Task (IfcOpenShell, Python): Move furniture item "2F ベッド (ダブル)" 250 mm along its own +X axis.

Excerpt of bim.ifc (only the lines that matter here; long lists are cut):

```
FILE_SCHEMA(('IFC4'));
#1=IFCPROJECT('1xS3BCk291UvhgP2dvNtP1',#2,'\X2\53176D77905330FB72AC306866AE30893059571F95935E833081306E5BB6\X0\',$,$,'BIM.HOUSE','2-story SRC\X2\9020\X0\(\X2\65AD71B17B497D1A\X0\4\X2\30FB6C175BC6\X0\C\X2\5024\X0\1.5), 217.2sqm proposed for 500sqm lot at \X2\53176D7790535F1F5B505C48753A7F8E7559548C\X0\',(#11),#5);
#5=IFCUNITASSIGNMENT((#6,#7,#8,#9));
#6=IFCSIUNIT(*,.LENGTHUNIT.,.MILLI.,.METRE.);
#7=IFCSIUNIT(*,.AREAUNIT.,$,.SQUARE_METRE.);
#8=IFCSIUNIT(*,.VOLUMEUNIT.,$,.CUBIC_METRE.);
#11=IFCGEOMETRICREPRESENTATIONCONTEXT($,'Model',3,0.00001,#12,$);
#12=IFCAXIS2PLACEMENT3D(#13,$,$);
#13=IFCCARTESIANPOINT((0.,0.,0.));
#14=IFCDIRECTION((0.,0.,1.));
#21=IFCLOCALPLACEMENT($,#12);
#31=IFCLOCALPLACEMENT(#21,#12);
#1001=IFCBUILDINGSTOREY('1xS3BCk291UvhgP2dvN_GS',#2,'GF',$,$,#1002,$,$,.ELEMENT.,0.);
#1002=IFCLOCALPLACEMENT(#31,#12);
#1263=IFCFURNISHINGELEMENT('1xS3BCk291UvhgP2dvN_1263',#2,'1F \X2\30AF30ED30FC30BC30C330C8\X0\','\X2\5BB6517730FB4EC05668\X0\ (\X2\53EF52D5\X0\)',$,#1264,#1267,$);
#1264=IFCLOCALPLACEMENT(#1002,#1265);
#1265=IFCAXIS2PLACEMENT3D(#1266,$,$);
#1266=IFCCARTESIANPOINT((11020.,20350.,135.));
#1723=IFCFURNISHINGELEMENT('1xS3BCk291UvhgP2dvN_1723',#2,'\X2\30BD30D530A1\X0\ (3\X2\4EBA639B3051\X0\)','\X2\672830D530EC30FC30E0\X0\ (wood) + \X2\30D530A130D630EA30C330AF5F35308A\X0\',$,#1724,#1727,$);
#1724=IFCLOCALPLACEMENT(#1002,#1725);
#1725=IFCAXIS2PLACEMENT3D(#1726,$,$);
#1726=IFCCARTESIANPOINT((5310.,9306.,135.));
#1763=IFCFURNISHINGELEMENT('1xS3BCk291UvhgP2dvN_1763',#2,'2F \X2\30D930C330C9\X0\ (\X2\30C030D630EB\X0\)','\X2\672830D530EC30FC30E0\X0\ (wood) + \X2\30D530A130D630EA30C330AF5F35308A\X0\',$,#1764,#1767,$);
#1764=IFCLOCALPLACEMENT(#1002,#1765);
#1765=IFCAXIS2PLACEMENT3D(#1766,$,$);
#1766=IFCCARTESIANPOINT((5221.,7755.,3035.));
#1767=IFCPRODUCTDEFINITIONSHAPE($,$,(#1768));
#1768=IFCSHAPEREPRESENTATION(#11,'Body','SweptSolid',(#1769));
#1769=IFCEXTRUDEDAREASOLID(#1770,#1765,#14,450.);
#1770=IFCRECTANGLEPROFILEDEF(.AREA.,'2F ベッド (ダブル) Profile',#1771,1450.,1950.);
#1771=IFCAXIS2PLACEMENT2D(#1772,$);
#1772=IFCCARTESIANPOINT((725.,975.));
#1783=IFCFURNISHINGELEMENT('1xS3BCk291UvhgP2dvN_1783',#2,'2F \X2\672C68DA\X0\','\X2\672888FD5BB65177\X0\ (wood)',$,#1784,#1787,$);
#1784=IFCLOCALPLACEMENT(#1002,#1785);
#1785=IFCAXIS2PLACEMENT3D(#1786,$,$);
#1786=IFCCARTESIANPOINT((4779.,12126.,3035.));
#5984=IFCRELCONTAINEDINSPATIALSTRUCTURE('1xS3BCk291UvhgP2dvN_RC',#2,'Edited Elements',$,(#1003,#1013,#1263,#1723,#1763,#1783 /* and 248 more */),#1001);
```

```python
import ifcopenshell
import ifcopenshell.api.geometry
import ifcopenshell.util.placement

model = ifcopenshell.open("bim.ifc")

item = model.by_guid("1xS3BCk291UvhgP2dvN_1763")
matrix = ifcopenshell.util.placement.get_local_placement(item.ObjectPlacement)
matrix[:3, 3] += matrix[:3, 0] * 250.0
ifcopenshell.api.geometry.edit_object_placement(model, product=item, matrix=matrix, is_si=False)

print(ifcopenshell.util.placement.get_local_placement(item.ObjectPlacement).round(3) + 0.0)

model.write("bim-out.ifc")
```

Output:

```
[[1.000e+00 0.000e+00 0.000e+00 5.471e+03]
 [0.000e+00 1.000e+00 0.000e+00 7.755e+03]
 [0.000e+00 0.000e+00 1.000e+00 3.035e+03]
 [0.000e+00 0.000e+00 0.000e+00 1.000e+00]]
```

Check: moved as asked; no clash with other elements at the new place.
